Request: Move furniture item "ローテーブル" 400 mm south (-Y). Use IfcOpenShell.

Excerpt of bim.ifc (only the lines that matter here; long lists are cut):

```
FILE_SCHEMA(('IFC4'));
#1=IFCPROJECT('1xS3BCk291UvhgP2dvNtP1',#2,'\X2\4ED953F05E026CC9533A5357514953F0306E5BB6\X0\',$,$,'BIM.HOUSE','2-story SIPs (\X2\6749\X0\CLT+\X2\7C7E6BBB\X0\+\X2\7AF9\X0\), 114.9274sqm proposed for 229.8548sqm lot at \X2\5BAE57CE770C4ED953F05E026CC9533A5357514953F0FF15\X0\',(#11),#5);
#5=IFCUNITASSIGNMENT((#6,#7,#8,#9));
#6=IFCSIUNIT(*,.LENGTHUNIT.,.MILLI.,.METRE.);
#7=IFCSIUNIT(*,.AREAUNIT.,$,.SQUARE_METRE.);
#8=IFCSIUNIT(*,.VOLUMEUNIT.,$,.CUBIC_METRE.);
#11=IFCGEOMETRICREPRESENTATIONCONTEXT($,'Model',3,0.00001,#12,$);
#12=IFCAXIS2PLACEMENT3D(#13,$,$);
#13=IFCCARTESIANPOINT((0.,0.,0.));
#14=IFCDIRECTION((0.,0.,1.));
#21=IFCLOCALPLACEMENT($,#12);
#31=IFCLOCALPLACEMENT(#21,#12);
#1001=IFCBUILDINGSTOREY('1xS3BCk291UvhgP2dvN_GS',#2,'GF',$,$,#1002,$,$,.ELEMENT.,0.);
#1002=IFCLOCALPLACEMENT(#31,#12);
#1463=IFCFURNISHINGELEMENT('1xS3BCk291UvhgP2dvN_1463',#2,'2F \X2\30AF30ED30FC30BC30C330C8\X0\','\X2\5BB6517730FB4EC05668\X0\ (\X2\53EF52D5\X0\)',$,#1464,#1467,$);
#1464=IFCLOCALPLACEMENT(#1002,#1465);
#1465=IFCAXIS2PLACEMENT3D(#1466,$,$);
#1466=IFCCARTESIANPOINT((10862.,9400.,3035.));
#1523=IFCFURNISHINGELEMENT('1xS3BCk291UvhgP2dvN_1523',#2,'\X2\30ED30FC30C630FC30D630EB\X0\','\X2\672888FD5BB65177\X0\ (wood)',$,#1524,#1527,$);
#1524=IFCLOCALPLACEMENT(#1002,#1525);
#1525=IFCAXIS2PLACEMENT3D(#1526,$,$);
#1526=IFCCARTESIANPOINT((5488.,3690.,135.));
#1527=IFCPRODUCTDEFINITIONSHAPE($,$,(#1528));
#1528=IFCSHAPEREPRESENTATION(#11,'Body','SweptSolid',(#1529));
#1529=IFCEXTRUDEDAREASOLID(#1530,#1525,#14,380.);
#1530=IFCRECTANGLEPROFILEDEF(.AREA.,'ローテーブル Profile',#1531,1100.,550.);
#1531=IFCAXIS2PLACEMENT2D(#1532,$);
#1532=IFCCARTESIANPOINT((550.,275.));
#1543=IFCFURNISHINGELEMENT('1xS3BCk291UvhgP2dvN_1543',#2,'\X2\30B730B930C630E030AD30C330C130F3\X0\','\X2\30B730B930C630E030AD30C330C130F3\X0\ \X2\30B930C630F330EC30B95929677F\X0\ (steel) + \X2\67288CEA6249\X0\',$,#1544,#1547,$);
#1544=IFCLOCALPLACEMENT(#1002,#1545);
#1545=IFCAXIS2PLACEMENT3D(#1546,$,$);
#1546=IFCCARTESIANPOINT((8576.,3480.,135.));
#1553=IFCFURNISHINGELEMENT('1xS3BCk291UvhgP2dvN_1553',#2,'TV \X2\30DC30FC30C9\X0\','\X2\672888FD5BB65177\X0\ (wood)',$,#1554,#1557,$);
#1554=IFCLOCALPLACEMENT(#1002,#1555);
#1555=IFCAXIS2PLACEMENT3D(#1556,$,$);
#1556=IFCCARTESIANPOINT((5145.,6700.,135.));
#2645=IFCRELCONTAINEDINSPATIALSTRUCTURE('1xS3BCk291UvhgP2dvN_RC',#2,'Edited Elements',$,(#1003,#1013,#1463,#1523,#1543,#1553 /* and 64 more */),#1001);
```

```python
import ifcopenshell
import ifcopenshell.api.geometry
import ifcopenshell.util.placement
import ifcopenshell.util.unit

model = ifcopenshell.open("bim.ifc")
unit_scale = ifcopenshell.util.unit.calculate_unit_scale(model)

item = model.by_guid("1xS3BCk291UvhgP2dvN_1523")
matrix = ifcopenshell.util.placement.get_local_placement(item.ObjectPlacement)
matrix[1, 3] -= 0.4 / unit_scale
ifcopenshell.api.geometry.edit_object_placement(model, product=item, matrix=matrix, is_si=False)

print(ifcopenshell.util.placement.get_local_placement(item.ObjectPlacement).round(3) + 0.0)

model.write("bim_v2.ifc")
```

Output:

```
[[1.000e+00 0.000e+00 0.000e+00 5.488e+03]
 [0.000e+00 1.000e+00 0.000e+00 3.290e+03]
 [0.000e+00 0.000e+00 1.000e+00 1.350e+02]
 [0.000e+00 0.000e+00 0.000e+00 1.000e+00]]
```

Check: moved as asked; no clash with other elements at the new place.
